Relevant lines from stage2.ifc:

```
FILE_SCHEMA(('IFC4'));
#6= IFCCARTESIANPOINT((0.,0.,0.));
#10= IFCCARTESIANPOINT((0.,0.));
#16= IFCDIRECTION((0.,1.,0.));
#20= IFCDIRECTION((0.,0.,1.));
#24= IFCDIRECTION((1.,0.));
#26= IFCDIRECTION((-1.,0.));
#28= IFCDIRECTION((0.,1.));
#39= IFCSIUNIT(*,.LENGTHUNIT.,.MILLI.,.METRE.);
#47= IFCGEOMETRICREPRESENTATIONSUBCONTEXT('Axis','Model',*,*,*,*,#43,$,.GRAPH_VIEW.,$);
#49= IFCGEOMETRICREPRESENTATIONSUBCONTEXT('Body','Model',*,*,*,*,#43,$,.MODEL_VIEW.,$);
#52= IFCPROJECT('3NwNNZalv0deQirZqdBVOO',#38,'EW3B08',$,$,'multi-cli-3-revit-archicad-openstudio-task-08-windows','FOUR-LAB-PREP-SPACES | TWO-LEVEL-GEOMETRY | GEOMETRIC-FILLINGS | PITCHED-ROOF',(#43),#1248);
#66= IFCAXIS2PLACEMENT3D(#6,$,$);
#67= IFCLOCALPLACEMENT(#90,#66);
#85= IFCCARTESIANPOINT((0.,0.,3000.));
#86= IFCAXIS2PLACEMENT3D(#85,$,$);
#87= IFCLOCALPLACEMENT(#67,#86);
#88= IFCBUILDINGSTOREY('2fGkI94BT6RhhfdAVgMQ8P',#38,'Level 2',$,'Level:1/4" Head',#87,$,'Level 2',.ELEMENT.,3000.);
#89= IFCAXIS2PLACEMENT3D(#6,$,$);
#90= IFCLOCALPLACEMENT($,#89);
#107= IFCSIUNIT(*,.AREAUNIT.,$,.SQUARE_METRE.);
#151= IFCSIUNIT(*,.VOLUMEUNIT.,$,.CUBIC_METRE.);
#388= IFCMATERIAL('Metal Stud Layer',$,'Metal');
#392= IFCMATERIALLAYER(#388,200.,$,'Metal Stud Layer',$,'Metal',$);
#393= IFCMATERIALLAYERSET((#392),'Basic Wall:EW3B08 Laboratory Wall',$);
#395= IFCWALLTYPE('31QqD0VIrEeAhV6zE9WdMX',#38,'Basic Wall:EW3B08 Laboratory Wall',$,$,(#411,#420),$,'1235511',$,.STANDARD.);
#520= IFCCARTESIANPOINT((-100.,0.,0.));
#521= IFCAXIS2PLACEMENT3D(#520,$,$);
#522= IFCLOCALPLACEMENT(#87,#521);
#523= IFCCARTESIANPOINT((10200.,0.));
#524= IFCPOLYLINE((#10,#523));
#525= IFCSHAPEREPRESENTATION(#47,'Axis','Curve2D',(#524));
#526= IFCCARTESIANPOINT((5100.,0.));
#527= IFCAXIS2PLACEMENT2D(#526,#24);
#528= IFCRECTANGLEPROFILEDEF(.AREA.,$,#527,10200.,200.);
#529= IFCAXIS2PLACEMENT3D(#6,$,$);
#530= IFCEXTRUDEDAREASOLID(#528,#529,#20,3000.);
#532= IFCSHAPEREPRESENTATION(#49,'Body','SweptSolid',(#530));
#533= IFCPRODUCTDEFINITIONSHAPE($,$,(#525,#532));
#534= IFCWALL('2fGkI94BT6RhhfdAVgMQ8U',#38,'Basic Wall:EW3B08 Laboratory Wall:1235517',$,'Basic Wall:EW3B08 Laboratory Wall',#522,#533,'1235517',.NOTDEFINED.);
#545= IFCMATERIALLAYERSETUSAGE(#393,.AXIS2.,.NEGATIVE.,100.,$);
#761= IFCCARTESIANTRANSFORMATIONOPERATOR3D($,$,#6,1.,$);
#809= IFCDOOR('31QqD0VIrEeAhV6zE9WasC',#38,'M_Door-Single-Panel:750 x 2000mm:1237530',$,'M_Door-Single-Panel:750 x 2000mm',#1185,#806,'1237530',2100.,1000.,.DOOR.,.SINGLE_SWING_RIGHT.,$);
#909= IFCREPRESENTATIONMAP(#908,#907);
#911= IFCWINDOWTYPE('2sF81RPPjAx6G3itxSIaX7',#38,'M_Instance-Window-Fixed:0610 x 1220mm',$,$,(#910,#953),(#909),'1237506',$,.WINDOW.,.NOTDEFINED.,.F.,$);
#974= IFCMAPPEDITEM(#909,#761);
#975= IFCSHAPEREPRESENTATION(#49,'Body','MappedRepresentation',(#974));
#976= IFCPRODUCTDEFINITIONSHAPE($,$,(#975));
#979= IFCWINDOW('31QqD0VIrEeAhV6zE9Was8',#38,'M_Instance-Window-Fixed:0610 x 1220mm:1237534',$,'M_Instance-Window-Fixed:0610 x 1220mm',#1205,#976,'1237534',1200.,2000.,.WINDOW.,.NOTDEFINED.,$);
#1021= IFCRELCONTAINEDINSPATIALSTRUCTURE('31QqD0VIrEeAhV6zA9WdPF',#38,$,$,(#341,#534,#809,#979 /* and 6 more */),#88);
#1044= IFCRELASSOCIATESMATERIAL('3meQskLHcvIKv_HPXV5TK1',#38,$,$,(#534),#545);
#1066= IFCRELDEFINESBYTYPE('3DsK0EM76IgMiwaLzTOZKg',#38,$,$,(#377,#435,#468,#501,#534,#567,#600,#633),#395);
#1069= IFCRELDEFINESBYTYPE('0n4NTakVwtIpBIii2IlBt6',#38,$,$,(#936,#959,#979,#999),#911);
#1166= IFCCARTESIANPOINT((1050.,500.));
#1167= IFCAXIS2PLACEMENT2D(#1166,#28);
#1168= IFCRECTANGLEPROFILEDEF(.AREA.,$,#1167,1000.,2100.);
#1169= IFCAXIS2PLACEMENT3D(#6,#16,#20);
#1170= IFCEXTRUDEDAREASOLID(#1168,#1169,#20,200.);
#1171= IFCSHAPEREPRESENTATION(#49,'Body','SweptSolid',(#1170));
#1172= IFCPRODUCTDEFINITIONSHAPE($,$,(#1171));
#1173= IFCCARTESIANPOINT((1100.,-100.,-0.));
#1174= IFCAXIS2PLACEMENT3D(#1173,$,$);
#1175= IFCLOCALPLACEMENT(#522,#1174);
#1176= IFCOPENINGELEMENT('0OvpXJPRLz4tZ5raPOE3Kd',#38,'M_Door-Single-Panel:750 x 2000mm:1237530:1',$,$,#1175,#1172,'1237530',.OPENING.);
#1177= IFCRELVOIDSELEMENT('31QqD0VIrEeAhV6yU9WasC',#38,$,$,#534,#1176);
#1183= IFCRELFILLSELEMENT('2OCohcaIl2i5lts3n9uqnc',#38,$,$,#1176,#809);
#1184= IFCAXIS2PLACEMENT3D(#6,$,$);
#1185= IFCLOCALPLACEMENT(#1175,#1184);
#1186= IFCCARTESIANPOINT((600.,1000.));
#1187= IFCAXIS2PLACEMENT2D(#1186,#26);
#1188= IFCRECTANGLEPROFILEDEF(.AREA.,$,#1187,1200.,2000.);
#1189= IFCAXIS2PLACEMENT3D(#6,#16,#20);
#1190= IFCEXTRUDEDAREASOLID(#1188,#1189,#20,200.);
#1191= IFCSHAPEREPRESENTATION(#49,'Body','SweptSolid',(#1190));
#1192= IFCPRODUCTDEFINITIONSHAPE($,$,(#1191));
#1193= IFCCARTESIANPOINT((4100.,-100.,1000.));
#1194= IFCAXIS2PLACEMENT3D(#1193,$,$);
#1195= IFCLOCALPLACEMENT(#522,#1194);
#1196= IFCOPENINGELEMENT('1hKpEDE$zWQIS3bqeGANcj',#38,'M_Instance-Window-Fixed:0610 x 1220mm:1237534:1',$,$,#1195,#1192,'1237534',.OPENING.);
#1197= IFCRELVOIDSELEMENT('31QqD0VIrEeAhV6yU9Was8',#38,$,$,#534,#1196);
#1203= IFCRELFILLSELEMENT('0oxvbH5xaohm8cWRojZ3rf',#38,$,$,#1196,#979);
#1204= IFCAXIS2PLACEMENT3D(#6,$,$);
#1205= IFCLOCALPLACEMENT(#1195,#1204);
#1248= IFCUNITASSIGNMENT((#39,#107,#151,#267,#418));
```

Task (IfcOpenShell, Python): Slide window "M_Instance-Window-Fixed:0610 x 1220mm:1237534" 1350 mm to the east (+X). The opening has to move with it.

```python
import ifcopenshell
import ifcopenshell.api.geometry
import ifcopenshell.util.placement
import ifcopenshell.util.unit

model = ifcopenshell.open("stage2.ifc")
unit_scale = ifcopenshell.util.unit.calculate_unit_scale(model)

window = model.by_guid("31QqD0VIrEeAhV6zE9Was8")
opening = window.FillsVoids[0].RelatingOpeningElement
wall = opening.VoidsElements[0].RelatingBuildingElement

wall_matrix = ifcopenshell.util.placement.get_local_placement(wall.ObjectPlacement)
shift = wall_matrix[:3, 0] * 1.35 / unit_scale
before = ifcopenshell.util.placement.get_local_placement(window.ObjectPlacement)[:3, 3].copy()

# The window is placed relative to its opening, so it follows when the opening moves.
matrix = ifcopenshell.util.placement.get_local_placement(opening.ObjectPlacement)
matrix[:3, 3] += shift
ifcopenshell.api.geometry.edit_object_placement(
    model, product=opening, matrix=matrix, is_si=False, should_transform_children=True
)

after = ifcopenshell.util.placement.get_local_placement(window.ObjectPlacement)[:3, 3]
print("window moved by", (after - before).round(3) + 0.0)

model.write("stage2_rev.ifc")
```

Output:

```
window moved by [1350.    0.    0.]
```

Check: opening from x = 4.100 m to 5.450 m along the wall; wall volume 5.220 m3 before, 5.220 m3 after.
